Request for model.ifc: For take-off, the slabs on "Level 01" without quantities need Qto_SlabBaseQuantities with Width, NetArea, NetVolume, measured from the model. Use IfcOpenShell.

First a look at what the model holds.

```python
import ifcopenshell
import ifcopenshell.util.element
import ifcopenshell.util.unit

model = ifcopenshell.open("model.ifc")
print(model.schema)
for unit_type in ("LENGTHUNIT", "AREAUNIT", "VOLUMEUNIT"):
    print(unit_type, ifcopenshell.util.unit.calculate_unit_scale(model, unit_type))
storey = next(s for s in model.by_type("IfcBuildingStorey") if s.Name == "Level 01")
slabs = [e for e in ifcopenshell.util.element.get_decomposition(storey) if e.is_a("IfcSlab")]
for e in sorted(slabs, key=lambda e: e.id()):
    print(e.id(), e.is_a(), e.Name, list(ifcopenshell.util.element.get_psets(e, qtos_only=True)), sep=" | ")
```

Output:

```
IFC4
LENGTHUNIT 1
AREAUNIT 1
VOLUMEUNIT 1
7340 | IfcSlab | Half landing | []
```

```python
import ifcopenshell
import ifcopenshell.api.pset
import ifcopenshell.geom
import ifcopenshell.util.element
import ifcopenshell.util.shape
import ifcopenshell.util.unit

model = ifcopenshell.open("model.ifc")
unit_scale = ifcopenshell.util.unit.calculate_unit_scale(model)
area_scale = ifcopenshell.util.unit.calculate_unit_scale(model, "AREAUNIT")
volume_scale = ifcopenshell.util.unit.calculate_unit_scale(model, "VOLUMEUNIT")
settings = ifcopenshell.geom.settings()

storey = next(s for s in model.by_type("IfcBuildingStorey") if s.Name == "Level 01")
slabs = [e for e in ifcopenshell.util.element.get_decomposition(storey) if e.is_a("IfcSlab")]

for e in sorted(slabs, key=lambda e: e.id()):
    if ifcopenshell.util.element.get_psets(e, qtos_only=True, should_inherit=False):
        continue
    # Geometry comes back in metres, in the element's own axes.
    shape = ifcopenshell.geom.create_shape(settings, e)
    values = {
        "Width": ifcopenshell.util.shape.get_z(shape.geometry) / unit_scale,
        "NetArea": ifcopenshell.util.shape.get_footprint_area(shape.geometry) / area_scale,
        "NetVolume": ifcopenshell.util.shape.get_volume(shape.geometry) / volume_scale,
    }
    qto = ifcopenshell.api.pset.add_qto(model, product=e, name="Qto_SlabBaseQuantities")
    ifcopenshell.api.pset.edit_qto(model, qto=qto, properties=values)
    print(e.id(), {k: round(v, 3) for k, v in values.items()})

model.write("model_v2.ifc")
```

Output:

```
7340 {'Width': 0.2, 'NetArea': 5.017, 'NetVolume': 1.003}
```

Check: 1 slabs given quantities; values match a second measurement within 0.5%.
